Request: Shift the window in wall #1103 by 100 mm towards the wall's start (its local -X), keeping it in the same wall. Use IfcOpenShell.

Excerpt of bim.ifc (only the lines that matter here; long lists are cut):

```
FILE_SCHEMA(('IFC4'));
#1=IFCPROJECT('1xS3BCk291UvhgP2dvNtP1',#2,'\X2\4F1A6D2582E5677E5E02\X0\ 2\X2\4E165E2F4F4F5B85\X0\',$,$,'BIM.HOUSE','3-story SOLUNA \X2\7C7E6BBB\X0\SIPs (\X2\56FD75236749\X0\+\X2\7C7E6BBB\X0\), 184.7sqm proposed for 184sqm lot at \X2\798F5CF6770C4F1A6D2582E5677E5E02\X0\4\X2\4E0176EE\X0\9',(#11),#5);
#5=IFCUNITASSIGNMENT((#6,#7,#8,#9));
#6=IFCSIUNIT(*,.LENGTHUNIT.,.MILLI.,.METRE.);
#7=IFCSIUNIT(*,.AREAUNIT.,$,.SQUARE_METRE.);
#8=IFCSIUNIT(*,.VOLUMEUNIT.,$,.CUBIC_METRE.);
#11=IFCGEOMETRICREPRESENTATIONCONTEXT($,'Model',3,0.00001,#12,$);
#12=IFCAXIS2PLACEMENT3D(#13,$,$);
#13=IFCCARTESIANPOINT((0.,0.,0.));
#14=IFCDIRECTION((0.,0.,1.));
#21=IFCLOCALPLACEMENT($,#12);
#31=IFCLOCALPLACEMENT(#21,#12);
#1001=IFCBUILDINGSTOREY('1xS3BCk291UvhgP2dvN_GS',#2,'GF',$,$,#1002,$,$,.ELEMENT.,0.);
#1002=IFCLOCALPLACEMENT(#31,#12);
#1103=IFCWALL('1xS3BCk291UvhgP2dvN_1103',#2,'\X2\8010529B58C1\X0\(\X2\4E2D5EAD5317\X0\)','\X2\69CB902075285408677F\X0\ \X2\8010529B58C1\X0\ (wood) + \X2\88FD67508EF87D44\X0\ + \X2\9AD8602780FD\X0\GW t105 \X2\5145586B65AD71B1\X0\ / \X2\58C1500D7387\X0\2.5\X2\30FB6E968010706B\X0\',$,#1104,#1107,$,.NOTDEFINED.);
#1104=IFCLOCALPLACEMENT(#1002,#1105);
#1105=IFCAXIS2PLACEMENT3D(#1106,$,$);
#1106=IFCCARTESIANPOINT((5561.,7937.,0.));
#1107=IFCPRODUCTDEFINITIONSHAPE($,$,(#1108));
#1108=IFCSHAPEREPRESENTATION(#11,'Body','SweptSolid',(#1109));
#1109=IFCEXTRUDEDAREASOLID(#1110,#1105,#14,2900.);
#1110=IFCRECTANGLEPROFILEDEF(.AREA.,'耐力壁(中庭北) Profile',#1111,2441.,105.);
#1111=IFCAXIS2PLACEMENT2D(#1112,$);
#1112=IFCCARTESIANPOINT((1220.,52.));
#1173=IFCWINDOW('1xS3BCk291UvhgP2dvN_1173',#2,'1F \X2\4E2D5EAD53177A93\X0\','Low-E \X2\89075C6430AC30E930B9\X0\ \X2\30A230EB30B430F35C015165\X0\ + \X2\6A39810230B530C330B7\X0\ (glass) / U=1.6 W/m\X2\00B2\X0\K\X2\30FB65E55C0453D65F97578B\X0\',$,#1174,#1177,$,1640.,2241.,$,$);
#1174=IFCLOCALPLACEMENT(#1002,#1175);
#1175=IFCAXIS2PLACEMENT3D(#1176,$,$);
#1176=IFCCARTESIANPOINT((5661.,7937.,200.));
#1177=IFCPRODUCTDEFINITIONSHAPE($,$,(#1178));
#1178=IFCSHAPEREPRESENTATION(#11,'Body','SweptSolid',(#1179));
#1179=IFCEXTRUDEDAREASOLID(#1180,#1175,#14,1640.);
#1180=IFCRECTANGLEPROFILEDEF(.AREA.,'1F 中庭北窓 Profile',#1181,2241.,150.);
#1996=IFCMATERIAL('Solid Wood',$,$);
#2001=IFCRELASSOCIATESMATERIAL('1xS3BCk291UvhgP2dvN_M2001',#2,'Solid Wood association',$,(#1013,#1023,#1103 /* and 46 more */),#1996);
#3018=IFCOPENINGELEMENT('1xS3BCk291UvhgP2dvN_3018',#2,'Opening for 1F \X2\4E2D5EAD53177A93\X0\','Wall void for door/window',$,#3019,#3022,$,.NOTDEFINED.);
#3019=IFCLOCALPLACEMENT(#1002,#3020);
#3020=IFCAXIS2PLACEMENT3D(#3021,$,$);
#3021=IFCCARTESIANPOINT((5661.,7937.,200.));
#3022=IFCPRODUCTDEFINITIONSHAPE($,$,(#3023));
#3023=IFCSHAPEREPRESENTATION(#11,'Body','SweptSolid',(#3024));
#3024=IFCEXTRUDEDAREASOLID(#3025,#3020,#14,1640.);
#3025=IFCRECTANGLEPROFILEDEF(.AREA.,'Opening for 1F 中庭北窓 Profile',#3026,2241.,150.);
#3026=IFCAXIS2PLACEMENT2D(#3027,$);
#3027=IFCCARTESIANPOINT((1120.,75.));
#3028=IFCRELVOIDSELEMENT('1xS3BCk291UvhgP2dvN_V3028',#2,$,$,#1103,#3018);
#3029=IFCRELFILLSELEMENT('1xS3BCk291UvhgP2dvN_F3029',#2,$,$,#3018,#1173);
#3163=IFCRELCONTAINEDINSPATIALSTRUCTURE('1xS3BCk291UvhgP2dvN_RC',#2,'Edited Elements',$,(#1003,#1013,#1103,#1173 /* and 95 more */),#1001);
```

```python
import ifcopenshell
import ifcopenshell.api.geometry
import ifcopenshell.util.placement
import ifcopenshell.util.unit

model = ifcopenshell.open("bim.ifc")
unit_scale = ifcopenshell.util.unit.calculate_unit_scale(model)

window = model.by_guid("1xS3BCk291UvhgP2dvN_1173")
opening = window.FillsVoids[0].RelatingOpeningElement
wall = opening.VoidsElements[0].RelatingBuildingElement

wall_matrix = ifcopenshell.util.placement.get_local_placement(wall.ObjectPlacement)
shift = wall_matrix[:3, 0] * -0.1 / unit_scale
before = ifcopenshell.util.placement.get_local_placement(window.ObjectPlacement)[:3, 3].copy()

# The window is not placed relative to its opening, so move both.
for product in (opening, window):
    matrix = ifcopenshell.util.placement.get_local_placement(product.ObjectPlacement)
    matrix[:3, 3] += shift
    ifcopenshell.api.geometry.edit_object_placement(model, product=product, matrix=matrix, is_si=False)

after = ifcopenshell.util.placement.get_local_placement(window.ObjectPlacement)[:3, 3]
print("window moved by", (after - before).round(3) + 0.0)

model.write("bim_v2.ifc")
```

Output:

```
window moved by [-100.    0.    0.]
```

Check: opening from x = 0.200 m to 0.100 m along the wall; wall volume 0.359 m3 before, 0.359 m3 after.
